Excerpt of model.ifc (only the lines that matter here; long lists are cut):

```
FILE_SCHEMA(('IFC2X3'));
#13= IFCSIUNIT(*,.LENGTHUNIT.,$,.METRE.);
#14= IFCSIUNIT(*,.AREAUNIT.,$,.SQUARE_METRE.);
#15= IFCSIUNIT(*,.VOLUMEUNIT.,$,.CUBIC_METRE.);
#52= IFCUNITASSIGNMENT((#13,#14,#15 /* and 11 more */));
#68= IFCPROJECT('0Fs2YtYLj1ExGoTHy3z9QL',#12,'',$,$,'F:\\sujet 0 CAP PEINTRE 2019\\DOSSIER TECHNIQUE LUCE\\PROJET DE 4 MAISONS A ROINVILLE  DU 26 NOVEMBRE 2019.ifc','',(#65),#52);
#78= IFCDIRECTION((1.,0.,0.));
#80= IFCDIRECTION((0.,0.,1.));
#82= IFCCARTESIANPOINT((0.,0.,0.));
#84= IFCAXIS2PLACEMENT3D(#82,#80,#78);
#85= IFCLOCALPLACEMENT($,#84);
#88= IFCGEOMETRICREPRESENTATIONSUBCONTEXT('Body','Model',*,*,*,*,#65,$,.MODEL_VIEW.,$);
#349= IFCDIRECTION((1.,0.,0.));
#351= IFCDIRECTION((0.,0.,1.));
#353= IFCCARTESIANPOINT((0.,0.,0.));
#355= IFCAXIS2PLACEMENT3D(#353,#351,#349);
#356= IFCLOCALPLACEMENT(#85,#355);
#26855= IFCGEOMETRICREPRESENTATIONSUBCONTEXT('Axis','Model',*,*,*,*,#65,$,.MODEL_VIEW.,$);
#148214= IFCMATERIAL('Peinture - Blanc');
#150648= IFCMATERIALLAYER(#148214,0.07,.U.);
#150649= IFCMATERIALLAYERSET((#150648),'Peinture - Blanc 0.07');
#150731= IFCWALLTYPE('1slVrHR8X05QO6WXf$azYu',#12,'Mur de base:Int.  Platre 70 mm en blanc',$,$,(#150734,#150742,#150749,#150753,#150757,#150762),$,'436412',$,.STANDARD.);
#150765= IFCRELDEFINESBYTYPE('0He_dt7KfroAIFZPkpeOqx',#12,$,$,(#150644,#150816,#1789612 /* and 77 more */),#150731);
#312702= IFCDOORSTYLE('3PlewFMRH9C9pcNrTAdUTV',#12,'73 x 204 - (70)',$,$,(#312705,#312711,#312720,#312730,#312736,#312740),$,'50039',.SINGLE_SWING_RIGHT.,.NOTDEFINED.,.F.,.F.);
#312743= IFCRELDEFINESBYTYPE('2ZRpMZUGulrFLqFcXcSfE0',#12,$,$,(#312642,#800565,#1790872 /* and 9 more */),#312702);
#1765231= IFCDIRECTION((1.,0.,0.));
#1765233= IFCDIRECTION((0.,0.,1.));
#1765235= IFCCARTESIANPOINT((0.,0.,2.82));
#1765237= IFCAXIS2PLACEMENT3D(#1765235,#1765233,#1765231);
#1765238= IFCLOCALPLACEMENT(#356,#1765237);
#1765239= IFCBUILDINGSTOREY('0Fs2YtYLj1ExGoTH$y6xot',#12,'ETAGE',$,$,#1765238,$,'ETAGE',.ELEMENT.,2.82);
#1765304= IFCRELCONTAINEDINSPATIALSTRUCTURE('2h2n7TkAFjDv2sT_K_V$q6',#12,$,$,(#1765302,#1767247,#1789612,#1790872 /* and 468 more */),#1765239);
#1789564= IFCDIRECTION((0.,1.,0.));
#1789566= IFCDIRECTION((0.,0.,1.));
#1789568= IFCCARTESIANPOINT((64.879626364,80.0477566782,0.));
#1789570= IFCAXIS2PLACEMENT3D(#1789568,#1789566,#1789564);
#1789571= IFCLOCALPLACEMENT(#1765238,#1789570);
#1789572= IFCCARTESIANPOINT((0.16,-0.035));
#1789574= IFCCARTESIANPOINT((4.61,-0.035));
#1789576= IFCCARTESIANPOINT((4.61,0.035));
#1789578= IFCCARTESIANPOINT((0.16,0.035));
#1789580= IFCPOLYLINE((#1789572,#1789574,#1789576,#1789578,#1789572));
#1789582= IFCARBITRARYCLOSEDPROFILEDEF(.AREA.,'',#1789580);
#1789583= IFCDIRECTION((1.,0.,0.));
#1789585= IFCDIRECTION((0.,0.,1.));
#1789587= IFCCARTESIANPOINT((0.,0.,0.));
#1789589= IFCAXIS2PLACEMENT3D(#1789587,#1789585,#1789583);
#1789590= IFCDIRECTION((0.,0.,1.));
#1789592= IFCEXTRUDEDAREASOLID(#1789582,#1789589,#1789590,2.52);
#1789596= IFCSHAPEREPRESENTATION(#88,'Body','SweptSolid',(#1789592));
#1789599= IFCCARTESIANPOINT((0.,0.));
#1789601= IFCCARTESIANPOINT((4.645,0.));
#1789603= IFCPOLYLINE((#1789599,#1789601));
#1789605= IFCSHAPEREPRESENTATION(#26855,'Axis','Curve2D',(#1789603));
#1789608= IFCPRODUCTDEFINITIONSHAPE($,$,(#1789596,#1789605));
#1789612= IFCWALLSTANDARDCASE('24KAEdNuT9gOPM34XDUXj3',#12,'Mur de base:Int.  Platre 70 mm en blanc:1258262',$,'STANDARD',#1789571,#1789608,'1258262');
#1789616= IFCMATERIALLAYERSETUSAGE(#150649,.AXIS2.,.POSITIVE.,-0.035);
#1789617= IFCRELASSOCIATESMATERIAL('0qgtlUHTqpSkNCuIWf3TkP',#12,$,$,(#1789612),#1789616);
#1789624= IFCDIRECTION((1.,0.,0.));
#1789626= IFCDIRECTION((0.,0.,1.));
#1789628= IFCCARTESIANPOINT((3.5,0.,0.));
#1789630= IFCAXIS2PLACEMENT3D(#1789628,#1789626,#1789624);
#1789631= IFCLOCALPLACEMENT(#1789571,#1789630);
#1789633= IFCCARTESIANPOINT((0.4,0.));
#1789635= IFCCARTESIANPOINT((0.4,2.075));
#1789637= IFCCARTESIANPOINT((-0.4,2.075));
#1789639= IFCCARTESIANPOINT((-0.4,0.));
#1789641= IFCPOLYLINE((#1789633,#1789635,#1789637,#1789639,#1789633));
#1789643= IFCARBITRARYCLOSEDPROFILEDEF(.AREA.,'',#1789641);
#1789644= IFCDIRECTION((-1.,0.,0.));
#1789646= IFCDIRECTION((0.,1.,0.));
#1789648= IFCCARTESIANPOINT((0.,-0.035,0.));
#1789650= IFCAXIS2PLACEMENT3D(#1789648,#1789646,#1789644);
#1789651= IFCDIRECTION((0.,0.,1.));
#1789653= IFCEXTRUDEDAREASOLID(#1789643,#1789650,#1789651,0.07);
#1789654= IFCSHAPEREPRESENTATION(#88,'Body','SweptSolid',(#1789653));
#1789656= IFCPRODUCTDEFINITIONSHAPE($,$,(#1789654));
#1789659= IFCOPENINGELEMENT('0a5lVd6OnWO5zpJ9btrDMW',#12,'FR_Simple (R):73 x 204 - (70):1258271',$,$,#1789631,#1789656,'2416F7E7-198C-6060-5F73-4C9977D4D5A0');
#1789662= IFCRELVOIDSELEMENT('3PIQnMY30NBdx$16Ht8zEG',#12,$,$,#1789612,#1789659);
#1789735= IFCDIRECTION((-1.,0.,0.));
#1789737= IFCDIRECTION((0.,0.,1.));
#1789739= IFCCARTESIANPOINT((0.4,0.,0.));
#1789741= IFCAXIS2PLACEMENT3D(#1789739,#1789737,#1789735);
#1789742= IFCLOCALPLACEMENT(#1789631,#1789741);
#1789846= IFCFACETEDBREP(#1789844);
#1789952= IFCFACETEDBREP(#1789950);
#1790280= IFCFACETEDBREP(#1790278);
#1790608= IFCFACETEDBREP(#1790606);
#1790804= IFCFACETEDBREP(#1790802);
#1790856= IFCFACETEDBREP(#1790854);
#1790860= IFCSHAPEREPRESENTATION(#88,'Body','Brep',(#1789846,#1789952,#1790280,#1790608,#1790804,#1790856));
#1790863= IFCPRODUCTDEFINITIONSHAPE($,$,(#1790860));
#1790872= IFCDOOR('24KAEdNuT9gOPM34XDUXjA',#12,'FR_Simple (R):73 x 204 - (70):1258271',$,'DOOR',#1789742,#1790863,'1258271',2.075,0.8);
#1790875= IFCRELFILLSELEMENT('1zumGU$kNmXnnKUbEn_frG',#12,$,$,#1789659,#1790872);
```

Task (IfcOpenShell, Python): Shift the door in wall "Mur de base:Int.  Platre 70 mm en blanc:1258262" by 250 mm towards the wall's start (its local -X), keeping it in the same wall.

```python
import ifcopenshell
import ifcopenshell.api.geometry
import ifcopenshell.util.placement
import ifcopenshell.util.unit

model = ifcopenshell.open("model.ifc")
unit_scale = ifcopenshell.util.unit.calculate_unit_scale(model)

door = model.by_guid("24KAEdNuT9gOPM34XDUXjA")
opening = door.FillsVoids[0].RelatingOpeningElement
wall = opening.VoidsElements[0].RelatingBuildingElement

wall_matrix = ifcopenshell.util.placement.get_local_placement(wall.ObjectPlacement)
shift = wall_matrix[:3, 0] * -0.25 / unit_scale
before = ifcopenshell.util.placement.get_local_placement(door.ObjectPlacement)[:3, 3].copy()

# The door is placed relative to its opening, so it follows when the opening moves.
matrix = ifcopenshell.util.placement.get_local_placement(opening.ObjectPlacement)
matrix[:3, 3] += shift
ifcopenshell.api.geometry.edit_object_placement(
    model, product=opening, matrix=matrix, is_si=False, should_transform_children=True
)

after = ifcopenshell.util.placement.get_local_placement(door.ObjectPlacement)[:3, 3]
print("door moved by", (after - before).round(3) + 0.0)

model.write("model_rev.ifc")
```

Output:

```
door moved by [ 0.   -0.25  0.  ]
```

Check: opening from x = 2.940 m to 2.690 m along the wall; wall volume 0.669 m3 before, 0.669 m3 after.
